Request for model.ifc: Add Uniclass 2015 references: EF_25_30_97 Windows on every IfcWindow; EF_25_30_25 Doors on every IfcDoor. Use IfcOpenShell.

First a look at what the model holds.

```python
import ifcopenshell

model = ifcopenshell.open("model.ifc")
print(model.schema)
print("classifications:", [c.Name for c in model.by_type("IfcClassification")])
for ifc_class in ("IfcDoor", "IfcRoof", "IfcStair", "IfcWall", "IfcWindow"):
    print(ifc_class, len(model.by_type(ifc_class)))
```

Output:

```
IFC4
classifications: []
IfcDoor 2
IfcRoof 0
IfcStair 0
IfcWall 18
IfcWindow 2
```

```python
import ifcopenshell
import ifcopenshell.api.classification

model = ifcopenshell.open("model.ifc")

system = ifcopenshell.api.classification.add_classification(model, classification="Uniclass 2015")

codes = {
    "IfcWindow": ("EF_25_30_97", "Windows"),
    "IfcDoor": ("EF_25_30_25", "Doors"),
}
for ifc_class, (code, name) in codes.items():
    products = model.by_type(ifc_class)
    ifcopenshell.api.classification.add_reference(
        model, products=products, classification=system, identification=code, name=name
    )
    print(code, len(products))

model.write("model_v2.ifc")
```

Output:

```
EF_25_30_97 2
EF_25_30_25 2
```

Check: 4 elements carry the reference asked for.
